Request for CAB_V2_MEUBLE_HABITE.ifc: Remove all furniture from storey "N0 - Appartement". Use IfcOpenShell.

First a look at what the model holds.

```python
import ifcopenshell
import ifcopenshell.util.element

model = ifcopenshell.open("CAB_V2_MEUBLE_HABITE.ifc")
print(model.schema)
storey = next(s for s in model.by_type("IfcBuildingStorey") if s.Name == "N0 - Appartement")
furniture = [e for e in ifcopenshell.util.element.get_decomposition(storey) if e.is_a("IfcFurnishingElement")]
seen = {}
for e in furniture:
    element_type = ifcopenshell.util.element.get_type(e)
    name = element_type.Name if element_type not in (None, e) else None
    seen[name] = seen.get(name, 0) + 1
for name, count in sorted(seen.items(), key=str):
    print(count, "x", name)
```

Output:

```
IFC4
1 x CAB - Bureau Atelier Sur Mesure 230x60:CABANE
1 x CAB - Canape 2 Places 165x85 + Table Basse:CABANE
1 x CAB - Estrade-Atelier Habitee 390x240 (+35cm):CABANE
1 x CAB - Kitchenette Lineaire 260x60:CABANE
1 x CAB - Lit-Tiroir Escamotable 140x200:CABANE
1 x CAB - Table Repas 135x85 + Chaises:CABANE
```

```python
import ifcopenshell
import ifcopenshell.api.root
import ifcopenshell.util.element

model = ifcopenshell.open("CAB_V2_MEUBLE_HABITE.ifc")

storey = next(s for s in model.by_type("IfcBuildingStorey") if s.Name == "N0 - Appartement")
furniture = [e for e in ifcopenshell.util.element.get_decomposition(storey) if e.is_a("IfcFurnishingElement")]

for e in furniture:
    ifcopenshell.api.root.remove_product(model, product=e)
print(len(furniture), "removed")

model.write("CAB_V2_MEUBLE_HABITE_updated.ifc")
```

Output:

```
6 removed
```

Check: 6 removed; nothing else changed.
